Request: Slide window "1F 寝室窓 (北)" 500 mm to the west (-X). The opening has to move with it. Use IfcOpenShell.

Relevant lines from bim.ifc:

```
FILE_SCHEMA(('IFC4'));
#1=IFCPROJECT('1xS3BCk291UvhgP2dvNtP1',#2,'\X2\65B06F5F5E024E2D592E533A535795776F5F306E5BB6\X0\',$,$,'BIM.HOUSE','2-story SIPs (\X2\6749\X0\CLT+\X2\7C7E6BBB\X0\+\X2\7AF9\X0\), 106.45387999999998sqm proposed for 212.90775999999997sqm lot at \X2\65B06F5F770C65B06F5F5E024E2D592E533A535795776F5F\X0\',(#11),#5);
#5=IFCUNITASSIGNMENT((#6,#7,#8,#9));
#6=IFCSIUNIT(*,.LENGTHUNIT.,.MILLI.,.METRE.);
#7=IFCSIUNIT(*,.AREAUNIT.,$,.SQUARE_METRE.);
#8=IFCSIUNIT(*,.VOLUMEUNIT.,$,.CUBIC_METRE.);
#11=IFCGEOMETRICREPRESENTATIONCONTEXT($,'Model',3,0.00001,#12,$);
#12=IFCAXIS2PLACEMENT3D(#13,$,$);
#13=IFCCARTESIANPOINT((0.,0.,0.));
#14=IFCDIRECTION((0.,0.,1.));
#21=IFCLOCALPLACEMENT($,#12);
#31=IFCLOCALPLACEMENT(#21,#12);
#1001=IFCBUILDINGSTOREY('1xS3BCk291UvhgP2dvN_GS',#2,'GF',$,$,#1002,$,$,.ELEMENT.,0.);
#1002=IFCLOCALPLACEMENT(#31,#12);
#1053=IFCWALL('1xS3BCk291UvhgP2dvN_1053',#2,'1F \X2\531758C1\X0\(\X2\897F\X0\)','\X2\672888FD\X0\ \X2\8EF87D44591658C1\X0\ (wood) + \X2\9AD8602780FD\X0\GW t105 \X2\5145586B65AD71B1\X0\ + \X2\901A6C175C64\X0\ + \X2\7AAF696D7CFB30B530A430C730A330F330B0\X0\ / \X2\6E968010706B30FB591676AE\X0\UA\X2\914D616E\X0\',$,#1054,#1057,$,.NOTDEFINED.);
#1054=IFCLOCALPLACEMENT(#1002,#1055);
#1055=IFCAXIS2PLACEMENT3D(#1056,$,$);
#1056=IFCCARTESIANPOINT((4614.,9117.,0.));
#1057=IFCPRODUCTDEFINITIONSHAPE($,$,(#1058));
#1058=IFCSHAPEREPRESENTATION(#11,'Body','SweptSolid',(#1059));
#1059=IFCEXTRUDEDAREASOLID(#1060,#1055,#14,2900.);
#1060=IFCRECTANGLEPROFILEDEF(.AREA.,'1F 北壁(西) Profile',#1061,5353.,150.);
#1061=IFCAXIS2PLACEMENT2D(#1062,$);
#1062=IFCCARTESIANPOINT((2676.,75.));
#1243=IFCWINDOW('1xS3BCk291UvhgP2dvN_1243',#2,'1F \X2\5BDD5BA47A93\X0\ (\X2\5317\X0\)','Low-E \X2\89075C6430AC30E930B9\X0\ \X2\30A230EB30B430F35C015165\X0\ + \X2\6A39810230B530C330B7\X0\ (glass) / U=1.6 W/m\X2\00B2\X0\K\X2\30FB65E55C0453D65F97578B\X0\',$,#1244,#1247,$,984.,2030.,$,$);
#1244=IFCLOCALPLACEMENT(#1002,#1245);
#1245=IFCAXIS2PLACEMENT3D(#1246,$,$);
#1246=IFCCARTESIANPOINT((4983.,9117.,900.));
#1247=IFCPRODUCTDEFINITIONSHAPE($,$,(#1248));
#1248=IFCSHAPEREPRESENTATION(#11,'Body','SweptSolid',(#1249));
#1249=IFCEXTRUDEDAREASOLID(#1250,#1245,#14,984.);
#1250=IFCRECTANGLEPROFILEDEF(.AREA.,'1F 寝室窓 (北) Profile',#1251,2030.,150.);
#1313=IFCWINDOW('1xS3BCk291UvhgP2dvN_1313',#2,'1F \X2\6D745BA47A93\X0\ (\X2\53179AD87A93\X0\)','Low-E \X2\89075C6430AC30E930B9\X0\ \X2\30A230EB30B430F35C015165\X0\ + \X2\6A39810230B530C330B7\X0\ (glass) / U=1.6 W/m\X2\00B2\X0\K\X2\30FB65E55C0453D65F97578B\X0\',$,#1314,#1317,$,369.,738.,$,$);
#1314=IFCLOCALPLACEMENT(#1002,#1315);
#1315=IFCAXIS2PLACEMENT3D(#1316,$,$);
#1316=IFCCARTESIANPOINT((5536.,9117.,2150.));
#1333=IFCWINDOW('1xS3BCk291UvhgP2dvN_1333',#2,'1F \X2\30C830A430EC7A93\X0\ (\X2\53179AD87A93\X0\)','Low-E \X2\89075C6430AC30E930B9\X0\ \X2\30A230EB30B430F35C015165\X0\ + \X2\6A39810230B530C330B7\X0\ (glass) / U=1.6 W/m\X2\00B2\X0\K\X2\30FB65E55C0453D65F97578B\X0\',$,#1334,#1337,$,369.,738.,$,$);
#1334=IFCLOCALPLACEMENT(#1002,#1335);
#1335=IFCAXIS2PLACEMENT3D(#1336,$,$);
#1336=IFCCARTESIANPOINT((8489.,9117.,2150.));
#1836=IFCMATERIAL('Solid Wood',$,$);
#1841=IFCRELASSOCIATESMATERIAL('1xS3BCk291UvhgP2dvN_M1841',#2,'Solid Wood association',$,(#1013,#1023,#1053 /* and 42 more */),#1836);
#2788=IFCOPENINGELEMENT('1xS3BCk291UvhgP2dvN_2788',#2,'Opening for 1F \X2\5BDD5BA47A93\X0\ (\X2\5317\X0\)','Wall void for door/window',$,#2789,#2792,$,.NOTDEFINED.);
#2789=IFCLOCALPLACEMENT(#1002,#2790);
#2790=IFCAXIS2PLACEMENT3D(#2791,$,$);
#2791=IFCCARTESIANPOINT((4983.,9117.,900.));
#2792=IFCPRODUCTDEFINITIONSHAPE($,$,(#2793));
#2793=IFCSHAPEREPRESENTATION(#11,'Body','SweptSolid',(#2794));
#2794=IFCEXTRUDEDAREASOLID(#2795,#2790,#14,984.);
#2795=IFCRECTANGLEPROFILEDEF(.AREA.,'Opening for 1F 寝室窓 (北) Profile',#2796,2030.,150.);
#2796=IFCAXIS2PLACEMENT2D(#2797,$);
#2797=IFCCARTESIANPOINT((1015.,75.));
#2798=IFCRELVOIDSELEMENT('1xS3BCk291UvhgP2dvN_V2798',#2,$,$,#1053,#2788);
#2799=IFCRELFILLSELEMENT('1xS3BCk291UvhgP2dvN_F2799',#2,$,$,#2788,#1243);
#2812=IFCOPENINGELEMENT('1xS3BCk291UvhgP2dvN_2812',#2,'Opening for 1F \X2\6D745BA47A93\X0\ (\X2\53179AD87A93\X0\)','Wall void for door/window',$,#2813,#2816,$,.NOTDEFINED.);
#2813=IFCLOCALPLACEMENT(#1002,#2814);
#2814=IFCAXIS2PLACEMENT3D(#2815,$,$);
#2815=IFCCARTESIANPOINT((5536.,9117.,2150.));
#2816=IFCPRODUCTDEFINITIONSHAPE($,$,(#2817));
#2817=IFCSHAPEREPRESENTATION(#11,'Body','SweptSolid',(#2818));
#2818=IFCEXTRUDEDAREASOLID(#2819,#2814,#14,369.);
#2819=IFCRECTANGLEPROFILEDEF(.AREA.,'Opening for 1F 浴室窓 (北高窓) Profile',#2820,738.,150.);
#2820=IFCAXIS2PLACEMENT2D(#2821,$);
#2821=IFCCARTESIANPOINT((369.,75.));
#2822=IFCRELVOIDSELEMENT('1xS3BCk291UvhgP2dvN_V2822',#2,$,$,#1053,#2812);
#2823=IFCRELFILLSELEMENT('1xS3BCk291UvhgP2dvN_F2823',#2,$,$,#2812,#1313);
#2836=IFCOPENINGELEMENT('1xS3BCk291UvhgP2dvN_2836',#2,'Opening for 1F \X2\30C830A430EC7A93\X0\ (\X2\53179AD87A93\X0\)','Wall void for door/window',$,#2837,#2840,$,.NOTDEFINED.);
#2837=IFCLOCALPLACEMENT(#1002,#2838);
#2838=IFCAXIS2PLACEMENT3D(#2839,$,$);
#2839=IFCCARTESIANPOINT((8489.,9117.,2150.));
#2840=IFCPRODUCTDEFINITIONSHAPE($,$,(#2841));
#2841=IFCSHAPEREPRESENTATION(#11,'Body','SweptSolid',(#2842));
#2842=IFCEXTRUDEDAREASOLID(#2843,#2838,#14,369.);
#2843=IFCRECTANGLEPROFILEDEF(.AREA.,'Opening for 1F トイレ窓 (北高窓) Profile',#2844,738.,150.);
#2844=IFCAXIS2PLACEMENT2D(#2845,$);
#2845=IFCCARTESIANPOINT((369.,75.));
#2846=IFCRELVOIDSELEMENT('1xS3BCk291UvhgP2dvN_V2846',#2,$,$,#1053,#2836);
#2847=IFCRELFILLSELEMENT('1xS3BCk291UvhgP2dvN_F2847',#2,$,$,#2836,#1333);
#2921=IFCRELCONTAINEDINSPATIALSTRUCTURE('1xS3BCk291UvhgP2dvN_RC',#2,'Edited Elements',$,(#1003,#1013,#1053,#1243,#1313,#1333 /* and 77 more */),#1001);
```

```python
import ifcopenshell
import ifcopenshell.api.geometry
import ifcopenshell.util.placement
import ifcopenshell.util.unit

model = ifcopenshell.open("bim.ifc")
unit_scale = ifcopenshell.util.unit.calculate_unit_scale(model)

window = model.by_guid("1xS3BCk291UvhgP2dvN_1243")
opening = window.FillsVoids[0].RelatingOpeningElement
wall = opening.VoidsElements[0].RelatingBuildingElement

wall_matrix = ifcopenshell.util.placement.get_local_placement(wall.ObjectPlacement)
shift = wall_matrix[:3, 0] * -0.5 / unit_scale
before = ifcopenshell.util.placement.get_local_placement(window.ObjectPlacement)[:3, 3].copy()

# The window is not placed relative to its opening, so move both.
for product in (opening, window):
    matrix = ifcopenshell.util.placement.get_local_placement(product.ObjectPlacement)
    matrix[:3, 3] += shift
    ifcopenshell.api.geometry.edit_object_placement(model, product=product, matrix=matrix, is_si=False)

after = ifcopenshell.util.placement.get_local_placement(window.ObjectPlacement)[:3, 3]
print("window moved by", (after - before).round(3) + 0.0)

model.write("bim_edited.ifc")
```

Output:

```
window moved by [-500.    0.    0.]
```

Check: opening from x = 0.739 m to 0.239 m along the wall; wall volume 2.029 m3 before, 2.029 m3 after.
